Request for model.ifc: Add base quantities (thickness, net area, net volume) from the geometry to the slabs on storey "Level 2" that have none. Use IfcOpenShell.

First a look at what the model holds.

```python
import ifcopenshell
import ifcopenshell.util.element
import ifcopenshell.util.unit

model = ifcopenshell.open("model.ifc")
print(model.schema)
for unit_type in ("LENGTHUNIT", "AREAUNIT", "VOLUMEUNIT"):
    print(unit_type, ifcopenshell.util.unit.calculate_unit_scale(model, unit_type))
storey = next(s for s in model.by_type("IfcBuildingStorey") if s.Name == "Level 2")
slabs = [e for e in ifcopenshell.util.element.get_decomposition(storey) if e.is_a("IfcSlab")]
for e in sorted(slabs, key=lambda e: e.id()):
    print(e.id(), e.is_a(), e.Name, list(ifcopenshell.util.element.get_psets(e, qtos_only=True)), sep=" | ")
```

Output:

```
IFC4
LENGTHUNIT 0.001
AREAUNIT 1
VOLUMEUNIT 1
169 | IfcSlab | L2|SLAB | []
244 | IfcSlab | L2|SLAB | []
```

```python
import ifcopenshell
import ifcopenshell.api.pset
import ifcopenshell.geom
import ifcopenshell.util.element
import ifcopenshell.util.shape
import ifcopenshell.util.unit

model = ifcopenshell.open("model.ifc")
unit_scale = ifcopenshell.util.unit.calculate_unit_scale(model)
area_scale = ifcopenshell.util.unit.calculate_unit_scale(model, "AREAUNIT")
volume_scale = ifcopenshell.util.unit.calculate_unit_scale(model, "VOLUMEUNIT")
settings = ifcopenshell.geom.settings()

storey = next(s for s in model.by_type("IfcBuildingStorey") if s.Name == "Level 2")
slabs = [e for e in ifcopenshell.util.element.get_decomposition(storey) if e.is_a("IfcSlab")]

for e in sorted(slabs, key=lambda e: e.id()):
    if ifcopenshell.util.element.get_psets(e, qtos_only=True, should_inherit=False):
        continue
    # Geometry comes back in metres, in the element's own axes.
    shape = ifcopenshell.geom.create_shape(settings, e)
    values = {
        "Width": ifcopenshell.util.shape.get_z(shape.geometry) / unit_scale,
        "NetArea": ifcopenshell.util.shape.get_footprint_area(shape.geometry) / area_scale,
        "NetVolume": ifcopenshell.util.shape.get_volume(shape.geometry) / volume_scale,
    }
    qto = ifcopenshell.api.pset.add_qto(model, product=e, name="Qto_SlabBaseQuantities")
    ifcopenshell.api.pset.edit_qto(model, qto=qto, properties=values)
    print(e.id(), {k: round(v, 3) for k, v in values.items()})

model.write("model_edited.ifc")
```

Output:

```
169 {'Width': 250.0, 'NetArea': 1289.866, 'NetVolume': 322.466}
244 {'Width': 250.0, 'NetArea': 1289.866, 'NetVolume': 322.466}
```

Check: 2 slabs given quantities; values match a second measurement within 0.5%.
